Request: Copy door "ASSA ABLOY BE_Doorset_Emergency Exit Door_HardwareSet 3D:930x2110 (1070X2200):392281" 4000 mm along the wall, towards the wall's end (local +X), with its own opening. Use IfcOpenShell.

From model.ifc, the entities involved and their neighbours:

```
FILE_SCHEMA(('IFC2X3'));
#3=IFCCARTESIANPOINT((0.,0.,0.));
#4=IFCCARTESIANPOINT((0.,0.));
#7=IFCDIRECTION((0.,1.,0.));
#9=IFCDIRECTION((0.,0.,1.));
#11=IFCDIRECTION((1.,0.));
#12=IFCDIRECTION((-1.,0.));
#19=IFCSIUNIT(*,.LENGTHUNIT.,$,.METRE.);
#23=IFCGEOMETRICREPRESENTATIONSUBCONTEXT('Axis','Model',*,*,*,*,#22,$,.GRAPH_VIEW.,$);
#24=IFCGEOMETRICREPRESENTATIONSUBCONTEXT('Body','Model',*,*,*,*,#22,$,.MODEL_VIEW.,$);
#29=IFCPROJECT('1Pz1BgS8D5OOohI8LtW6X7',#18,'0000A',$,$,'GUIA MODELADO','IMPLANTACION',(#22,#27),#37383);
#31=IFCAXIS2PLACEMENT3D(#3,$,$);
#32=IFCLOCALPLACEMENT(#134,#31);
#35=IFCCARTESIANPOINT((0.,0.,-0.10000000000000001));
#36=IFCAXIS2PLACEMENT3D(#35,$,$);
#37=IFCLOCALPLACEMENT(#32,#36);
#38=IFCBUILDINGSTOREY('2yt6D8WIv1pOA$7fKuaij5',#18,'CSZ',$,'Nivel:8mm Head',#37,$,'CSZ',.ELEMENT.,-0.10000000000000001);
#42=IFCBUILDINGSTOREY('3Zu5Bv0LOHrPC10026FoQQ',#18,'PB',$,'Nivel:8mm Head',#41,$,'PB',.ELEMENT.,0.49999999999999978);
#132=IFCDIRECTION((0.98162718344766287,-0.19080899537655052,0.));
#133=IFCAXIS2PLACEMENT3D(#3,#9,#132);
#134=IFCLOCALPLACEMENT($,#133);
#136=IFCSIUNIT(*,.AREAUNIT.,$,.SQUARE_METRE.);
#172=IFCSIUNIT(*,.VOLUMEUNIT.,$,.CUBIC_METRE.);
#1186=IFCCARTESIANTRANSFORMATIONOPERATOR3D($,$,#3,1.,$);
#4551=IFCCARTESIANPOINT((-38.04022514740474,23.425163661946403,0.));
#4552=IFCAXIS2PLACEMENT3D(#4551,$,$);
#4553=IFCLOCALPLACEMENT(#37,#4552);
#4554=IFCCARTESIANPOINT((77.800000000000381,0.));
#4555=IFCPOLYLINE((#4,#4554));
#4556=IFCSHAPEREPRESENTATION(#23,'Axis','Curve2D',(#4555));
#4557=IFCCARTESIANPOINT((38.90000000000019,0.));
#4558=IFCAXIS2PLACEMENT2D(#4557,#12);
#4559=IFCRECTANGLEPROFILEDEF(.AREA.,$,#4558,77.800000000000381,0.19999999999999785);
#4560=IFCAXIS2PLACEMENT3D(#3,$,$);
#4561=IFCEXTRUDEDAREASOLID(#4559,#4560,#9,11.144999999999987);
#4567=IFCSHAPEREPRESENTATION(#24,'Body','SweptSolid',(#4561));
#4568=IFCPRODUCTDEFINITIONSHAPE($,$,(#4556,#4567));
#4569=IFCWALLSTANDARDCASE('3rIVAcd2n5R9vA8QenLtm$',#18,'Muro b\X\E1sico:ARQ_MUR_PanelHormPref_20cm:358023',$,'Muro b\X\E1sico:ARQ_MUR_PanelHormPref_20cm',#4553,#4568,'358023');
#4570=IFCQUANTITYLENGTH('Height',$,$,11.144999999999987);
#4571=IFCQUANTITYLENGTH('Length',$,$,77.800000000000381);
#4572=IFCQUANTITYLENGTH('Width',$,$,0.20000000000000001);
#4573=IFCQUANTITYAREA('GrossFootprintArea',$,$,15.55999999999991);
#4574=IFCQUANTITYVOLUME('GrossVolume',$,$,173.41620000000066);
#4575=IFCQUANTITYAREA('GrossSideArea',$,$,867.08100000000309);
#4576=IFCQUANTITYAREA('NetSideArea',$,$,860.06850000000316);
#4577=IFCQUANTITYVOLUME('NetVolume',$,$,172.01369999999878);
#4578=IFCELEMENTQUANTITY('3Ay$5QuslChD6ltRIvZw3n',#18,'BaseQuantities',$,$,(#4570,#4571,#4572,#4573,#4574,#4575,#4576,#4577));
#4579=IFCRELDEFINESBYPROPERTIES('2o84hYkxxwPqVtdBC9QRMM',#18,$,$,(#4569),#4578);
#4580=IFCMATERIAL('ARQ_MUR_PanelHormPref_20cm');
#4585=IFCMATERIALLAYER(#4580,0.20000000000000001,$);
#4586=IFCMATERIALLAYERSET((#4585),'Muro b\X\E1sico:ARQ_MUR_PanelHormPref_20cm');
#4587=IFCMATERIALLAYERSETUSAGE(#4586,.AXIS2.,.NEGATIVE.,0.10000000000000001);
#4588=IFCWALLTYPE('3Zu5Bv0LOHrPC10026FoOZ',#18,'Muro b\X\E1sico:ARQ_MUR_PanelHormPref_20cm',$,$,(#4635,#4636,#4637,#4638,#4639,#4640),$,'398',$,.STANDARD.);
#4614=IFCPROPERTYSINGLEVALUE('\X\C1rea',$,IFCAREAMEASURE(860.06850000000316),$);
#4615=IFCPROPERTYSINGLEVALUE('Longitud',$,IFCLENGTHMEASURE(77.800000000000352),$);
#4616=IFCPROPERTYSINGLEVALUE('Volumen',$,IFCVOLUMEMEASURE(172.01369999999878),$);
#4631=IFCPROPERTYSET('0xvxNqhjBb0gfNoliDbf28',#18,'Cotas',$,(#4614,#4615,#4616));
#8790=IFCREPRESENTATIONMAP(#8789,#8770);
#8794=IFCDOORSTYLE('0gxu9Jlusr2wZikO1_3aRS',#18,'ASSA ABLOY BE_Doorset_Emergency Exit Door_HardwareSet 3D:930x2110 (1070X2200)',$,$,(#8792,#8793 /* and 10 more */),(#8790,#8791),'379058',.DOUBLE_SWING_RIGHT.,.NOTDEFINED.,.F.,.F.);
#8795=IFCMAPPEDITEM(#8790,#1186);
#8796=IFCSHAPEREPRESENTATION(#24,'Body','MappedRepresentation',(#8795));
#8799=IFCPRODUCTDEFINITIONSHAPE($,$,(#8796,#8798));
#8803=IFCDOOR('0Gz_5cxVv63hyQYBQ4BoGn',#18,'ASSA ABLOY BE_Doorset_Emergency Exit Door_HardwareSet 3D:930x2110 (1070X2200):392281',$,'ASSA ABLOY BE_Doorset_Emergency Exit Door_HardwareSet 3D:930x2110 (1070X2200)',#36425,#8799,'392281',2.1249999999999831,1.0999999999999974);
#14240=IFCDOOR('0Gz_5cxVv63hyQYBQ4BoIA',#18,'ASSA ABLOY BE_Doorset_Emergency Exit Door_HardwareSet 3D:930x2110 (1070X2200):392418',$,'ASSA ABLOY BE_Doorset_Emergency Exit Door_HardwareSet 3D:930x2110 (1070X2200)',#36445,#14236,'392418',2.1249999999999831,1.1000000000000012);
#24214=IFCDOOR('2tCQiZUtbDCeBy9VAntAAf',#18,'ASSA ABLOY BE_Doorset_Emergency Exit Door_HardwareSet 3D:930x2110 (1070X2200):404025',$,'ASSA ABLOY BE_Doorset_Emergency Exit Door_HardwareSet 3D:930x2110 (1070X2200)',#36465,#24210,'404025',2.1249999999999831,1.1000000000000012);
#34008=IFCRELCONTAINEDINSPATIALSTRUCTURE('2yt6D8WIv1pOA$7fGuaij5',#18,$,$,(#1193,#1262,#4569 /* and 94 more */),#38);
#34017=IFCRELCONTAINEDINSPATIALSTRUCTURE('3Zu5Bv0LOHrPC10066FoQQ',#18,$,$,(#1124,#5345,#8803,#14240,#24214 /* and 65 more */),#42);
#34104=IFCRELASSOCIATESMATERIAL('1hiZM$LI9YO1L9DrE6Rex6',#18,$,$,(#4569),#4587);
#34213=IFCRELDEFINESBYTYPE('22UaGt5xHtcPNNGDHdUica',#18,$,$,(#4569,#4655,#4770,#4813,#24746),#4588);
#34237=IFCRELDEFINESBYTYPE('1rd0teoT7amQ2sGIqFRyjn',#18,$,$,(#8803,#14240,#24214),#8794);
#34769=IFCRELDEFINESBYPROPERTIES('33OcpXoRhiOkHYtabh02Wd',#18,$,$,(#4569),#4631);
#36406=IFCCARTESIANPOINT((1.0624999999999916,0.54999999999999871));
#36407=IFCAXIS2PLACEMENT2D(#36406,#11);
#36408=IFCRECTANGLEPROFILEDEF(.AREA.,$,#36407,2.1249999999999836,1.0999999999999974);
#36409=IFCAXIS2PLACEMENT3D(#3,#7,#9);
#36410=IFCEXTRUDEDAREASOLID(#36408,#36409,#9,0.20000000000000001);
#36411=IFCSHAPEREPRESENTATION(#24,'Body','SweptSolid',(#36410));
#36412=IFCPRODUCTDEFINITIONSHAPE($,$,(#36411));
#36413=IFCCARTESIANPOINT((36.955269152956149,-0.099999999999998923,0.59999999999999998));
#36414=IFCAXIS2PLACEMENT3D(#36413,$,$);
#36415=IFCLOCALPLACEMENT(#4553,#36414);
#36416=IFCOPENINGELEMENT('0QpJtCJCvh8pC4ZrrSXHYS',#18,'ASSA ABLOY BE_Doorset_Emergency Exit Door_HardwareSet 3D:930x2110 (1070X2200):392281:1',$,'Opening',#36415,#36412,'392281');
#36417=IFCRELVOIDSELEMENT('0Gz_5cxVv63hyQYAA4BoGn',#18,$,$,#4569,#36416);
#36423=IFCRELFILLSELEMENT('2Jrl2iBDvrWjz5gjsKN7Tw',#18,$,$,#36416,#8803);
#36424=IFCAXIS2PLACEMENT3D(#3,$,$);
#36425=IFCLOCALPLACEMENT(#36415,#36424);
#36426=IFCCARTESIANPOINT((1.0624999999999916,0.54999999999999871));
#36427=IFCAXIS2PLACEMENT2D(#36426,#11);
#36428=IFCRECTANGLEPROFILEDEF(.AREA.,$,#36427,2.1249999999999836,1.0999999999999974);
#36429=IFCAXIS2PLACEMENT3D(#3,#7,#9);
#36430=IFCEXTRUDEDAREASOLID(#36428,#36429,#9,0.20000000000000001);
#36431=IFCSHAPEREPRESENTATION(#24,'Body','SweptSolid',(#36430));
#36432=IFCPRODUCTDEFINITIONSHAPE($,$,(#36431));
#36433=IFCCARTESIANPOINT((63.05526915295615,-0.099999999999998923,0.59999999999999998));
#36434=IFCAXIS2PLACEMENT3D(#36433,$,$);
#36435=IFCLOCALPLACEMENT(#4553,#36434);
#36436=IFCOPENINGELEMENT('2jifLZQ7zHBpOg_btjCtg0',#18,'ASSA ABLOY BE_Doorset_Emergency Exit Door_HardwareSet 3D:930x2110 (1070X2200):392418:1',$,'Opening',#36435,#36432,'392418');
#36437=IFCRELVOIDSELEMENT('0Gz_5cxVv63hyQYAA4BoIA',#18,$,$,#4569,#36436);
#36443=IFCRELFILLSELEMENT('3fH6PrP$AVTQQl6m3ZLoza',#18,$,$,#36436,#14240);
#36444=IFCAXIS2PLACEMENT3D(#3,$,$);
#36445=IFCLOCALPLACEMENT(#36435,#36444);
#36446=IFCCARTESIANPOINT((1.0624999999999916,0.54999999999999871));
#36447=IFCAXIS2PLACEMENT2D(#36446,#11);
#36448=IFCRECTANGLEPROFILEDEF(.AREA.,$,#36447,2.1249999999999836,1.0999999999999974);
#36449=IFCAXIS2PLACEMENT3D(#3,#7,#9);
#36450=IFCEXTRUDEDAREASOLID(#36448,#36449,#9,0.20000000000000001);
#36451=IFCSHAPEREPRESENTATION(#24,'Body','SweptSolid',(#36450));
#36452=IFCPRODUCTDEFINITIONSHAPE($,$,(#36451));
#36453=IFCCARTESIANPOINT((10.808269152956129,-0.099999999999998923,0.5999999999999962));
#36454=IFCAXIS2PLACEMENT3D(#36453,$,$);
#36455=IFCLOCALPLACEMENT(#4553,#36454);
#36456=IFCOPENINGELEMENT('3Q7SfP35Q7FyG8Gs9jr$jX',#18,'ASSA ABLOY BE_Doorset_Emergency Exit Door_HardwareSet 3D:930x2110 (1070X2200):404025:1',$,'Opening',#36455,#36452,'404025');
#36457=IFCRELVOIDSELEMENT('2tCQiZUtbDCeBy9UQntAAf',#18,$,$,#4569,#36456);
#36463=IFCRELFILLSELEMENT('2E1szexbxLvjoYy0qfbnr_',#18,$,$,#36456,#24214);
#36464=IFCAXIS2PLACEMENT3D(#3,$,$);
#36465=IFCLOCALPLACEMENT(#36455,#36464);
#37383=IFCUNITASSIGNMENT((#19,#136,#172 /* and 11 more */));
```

```python
import ifcopenshell
import ifcopenshell.api.feature
import ifcopenshell.api.geometry
import ifcopenshell.api.pset
import ifcopenshell.api.root
import ifcopenshell.geom
import ifcopenshell.util.element
import ifcopenshell.util.placement
import ifcopenshell.util.shape
import ifcopenshell.util.unit

model = ifcopenshell.open("model.ifc")
unit_scale = ifcopenshell.util.unit.calculate_unit_scale(model)
area_scale = ifcopenshell.util.unit.calculate_unit_scale(model, "AREAUNIT")
volume_scale = ifcopenshell.util.unit.calculate_unit_scale(model, "VOLUMEUNIT")
settings = ifcopenshell.geom.settings()


def volume(element):
    """Net volume in cubic metres, openings subtracted."""
    shape = ifcopenshell.geom.create_shape(settings, element)
    return ifcopenshell.util.shape.get_volume(shape.geometry)


def reuse_history(source, copy):
    """copy_class also copies each property set's owner history, people and application; keep the originals."""
    for rel in copy.IsDefinedBy:
        if rel.is_a("IfcRelDefinesByProperties") and (history := rel.RelatingPropertyDefinition.OwnerHistory):
            rel.RelatingPropertyDefinition.OwnerHistory = source.OwnerHistory
            ifcopenshell.util.element.remove_deep2(model, history)


door = model.by_id(8803)
opening = door.FillsVoids[0].RelatingOpeningElement
wall = opening.VoidsElements[0].RelatingBuildingElement
before = volume(wall)
shift = ifcopenshell.util.placement.get_local_placement(wall.ObjectPlacement)[:3, 0] * 4 / unit_scale

# copy_class copies the void relationship, type, container and properties, but no geometry.
new_opening = ifcopenshell.api.root.copy_class(model, product=opening)
new_opening.Representation = ifcopenshell.util.element.copy_deep(
    model, opening.Representation, exclude=["IfcGeometricRepresentationContext", "IfcRepresentationMap"]
)
new_opening.Name = "ASSA ABLOY BE_Doorset_Emergency Exit Door_HardwareSet 3D:930x2110 (1070X2200)"
new_opening.Tag = None
reuse_history(opening, new_opening)
new_door = ifcopenshell.api.root.copy_class(model, product=door)
new_door.Representation = ifcopenshell.util.element.copy_deep(
    model, door.Representation, exclude=["IfcGeometricRepresentationContext", "IfcRepresentationMap"]
)
new_door.Name = "ASSA ABLOY BE_Doorset_Emergency Exit Door_HardwareSet 3D:930x2110 (1070X2200)"
new_door.Tag = None
reuse_history(door, new_door)
fills = ifcopenshell.api.feature.add_filling(model, opening=new_opening, element=new_door)
fills.OwnerHistory = new_door.OwnerHistory  # required in IFC2X3

for old, new in ((opening, new_opening), (door, new_door)):
    matrix = ifcopenshell.util.placement.get_local_placement(old.ObjectPlacement)
    matrix[:3, 3] += shift
    ifcopenshell.api.geometry.edit_object_placement(model, product=new, matrix=matrix, is_si=False)

after = volume(wall)
thickness = 0.2  # wall thickness in metres

# Update the wall's stored quantities.
qto = model.by_id(ifcopenshell.util.element.get_pset(wall, "BaseQuantities", should_inherit=False)["id"])
ifcopenshell.api.pset.edit_qto(model, qto=qto, properties={
    "NetSideArea": after / thickness / area_scale,
    "NetVolume": after / volume_scale,
})
pset = model.by_id(ifcopenshell.util.element.get_pset(wall, "Cotas", should_inherit=False)["id"])
ifcopenshell.api.pset.edit_pset(model, pset=pset, properties={
    "Área": model.create_entity("IfcAreaMeasure", after / thickness / area_scale),
    "Volumen": model.create_entity("IfcVolumeMeasure", after / volume_scale),
})

print(f"wall volume {before:.3f} -> {after:.3f} m3")

model.write("model_edited.ifc")
```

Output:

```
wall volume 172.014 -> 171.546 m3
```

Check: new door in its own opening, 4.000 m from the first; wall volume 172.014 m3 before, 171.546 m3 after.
